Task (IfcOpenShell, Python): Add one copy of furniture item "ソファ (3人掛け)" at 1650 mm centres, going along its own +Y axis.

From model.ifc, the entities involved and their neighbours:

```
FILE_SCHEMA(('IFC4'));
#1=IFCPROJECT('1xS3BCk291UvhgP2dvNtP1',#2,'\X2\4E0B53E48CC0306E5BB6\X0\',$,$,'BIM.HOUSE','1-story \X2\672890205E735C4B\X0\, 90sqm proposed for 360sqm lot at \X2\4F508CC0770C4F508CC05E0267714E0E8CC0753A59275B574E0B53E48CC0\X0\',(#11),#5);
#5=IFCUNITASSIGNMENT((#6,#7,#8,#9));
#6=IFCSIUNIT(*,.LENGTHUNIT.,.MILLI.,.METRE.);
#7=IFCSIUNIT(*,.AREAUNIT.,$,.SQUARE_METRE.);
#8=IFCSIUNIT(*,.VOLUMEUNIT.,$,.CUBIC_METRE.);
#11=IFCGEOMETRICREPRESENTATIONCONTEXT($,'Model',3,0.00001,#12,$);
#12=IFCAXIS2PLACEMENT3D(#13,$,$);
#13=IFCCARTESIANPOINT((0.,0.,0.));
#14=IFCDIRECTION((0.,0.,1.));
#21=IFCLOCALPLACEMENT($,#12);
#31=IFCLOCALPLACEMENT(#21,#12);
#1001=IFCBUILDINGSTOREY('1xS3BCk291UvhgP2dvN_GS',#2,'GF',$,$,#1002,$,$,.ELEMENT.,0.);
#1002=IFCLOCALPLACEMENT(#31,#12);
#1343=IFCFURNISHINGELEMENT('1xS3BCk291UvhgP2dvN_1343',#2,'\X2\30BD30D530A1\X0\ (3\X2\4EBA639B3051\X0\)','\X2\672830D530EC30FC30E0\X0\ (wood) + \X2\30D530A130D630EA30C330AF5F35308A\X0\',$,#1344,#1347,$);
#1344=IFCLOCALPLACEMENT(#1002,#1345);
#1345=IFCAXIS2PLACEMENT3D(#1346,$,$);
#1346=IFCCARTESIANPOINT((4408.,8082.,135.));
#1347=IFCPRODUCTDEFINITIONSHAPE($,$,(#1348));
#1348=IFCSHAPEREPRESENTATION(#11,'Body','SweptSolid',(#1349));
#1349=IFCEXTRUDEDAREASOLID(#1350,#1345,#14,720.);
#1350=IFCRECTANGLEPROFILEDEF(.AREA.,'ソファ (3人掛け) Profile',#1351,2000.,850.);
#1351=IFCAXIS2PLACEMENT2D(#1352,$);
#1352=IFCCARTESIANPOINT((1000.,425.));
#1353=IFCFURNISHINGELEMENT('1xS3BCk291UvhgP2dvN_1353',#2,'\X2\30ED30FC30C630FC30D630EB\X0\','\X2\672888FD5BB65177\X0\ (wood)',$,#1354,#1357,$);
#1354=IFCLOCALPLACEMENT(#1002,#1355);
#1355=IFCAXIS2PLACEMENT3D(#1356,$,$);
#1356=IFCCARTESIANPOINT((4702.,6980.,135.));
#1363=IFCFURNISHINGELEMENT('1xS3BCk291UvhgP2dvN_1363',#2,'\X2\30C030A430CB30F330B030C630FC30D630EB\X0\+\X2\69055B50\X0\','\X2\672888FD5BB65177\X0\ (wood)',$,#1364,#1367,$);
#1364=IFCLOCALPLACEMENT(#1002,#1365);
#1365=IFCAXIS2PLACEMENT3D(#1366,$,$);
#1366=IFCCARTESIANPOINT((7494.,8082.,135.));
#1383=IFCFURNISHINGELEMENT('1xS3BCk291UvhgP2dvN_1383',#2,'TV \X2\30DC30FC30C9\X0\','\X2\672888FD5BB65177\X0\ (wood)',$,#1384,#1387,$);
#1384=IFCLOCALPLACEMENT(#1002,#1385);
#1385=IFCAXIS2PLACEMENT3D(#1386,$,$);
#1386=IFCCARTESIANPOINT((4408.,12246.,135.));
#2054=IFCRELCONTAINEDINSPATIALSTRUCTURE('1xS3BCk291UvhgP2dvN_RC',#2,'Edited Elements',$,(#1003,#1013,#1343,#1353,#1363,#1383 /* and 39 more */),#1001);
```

```python
import ifcopenshell
import ifcopenshell.api.geometry
import ifcopenshell.api.root
import ifcopenshell.util.element
import ifcopenshell.util.placement

model = ifcopenshell.open("model.ifc")


def reuse_history(source, copy):
    """copy_class also copies each property set's owner history, people and application; keep the originals."""
    for rel in copy.IsDefinedBy:
        if rel.is_a("IfcRelDefinesByProperties") and (history := rel.RelatingPropertyDefinition.OwnerHistory):
            rel.RelatingPropertyDefinition.OwnerHistory = source.OwnerHistory
            ifcopenshell.util.element.remove_deep2(model, history)


source = model.by_id(1343)
base = ifcopenshell.util.placement.get_local_placement(source.ObjectPlacement)
step = base[:3, 1] * 1650.0

for i in range(1, 2):
    copy = ifcopenshell.api.root.copy_class(model, product=source)
    copy.Representation = ifcopenshell.util.element.copy_deep(
        model, source.Representation, exclude=["IfcGeometricRepresentationContext", "IfcRepresentationMap"]
    )
    reuse_history(source, copy)
    matrix = base.copy()
    matrix[:3, 3] += i * step
    print("added at", matrix[:3, 3].round(3) + 0.0)
    ifcopenshell.api.geometry.edit_object_placement(model, product=copy, matrix=matrix, is_si=False)

model.write("model_rev.ifc")
```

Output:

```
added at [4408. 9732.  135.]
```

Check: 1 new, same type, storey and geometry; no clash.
